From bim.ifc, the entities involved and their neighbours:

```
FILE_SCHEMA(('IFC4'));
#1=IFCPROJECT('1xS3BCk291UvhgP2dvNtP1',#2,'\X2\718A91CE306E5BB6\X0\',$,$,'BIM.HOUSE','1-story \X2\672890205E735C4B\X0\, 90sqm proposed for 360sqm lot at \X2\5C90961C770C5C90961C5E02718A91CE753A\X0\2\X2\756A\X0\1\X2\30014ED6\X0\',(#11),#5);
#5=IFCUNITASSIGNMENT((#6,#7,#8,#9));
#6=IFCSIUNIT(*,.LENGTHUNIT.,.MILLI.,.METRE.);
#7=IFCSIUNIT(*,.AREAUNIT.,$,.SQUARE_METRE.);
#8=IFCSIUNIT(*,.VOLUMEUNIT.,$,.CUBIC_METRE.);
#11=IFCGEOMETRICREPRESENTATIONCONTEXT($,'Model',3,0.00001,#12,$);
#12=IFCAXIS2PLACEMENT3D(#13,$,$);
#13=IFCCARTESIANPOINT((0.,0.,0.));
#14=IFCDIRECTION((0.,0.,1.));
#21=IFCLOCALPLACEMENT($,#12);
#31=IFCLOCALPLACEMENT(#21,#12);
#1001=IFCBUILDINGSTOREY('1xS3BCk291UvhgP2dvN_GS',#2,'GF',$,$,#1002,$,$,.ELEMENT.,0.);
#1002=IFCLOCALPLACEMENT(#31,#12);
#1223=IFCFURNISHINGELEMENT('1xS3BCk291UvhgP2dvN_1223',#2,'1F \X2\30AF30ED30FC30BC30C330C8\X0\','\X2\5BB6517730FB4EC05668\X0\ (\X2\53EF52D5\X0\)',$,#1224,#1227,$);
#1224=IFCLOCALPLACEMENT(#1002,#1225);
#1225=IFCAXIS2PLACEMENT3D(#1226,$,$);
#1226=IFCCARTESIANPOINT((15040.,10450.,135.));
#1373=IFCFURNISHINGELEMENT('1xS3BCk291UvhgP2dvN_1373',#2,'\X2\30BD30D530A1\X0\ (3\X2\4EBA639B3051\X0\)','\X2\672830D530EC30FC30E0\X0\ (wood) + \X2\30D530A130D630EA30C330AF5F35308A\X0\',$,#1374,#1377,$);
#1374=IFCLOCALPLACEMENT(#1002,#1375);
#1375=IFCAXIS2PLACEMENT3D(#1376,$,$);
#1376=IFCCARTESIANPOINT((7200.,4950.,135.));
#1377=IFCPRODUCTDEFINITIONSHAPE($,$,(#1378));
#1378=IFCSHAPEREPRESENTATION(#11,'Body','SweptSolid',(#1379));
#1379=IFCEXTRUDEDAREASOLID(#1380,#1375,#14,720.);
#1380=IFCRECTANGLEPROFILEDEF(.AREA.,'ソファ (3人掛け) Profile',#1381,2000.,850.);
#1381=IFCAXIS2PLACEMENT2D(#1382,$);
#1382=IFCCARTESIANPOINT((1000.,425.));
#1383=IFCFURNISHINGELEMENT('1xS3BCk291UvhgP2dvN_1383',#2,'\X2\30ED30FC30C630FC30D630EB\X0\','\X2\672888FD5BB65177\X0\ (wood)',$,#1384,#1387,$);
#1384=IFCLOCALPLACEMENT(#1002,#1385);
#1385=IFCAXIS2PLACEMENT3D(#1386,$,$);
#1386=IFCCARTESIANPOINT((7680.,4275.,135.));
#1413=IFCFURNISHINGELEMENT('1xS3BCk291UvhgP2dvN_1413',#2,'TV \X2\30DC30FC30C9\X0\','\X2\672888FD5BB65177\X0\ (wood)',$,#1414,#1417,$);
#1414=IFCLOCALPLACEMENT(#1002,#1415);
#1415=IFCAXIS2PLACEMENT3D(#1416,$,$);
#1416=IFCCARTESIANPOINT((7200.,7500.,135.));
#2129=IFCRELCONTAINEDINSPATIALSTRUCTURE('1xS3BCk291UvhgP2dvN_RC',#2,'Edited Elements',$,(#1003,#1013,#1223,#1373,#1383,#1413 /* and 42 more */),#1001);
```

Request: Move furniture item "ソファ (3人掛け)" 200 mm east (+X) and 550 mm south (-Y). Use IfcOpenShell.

```python
import ifcopenshell
import ifcopenshell.api.geometry
import ifcopenshell.util.placement
import ifcopenshell.util.unit

model = ifcopenshell.open("bim.ifc")
unit_scale = ifcopenshell.util.unit.calculate_unit_scale(model)

item = model.by_guid("1xS3BCk291UvhgP2dvN_1373")
matrix = ifcopenshell.util.placement.get_local_placement(item.ObjectPlacement)
matrix[0, 3] += 0.2 / unit_scale
matrix[1, 3] -= 0.55 / unit_scale
ifcopenshell.api.geometry.edit_object_placement(model, product=item, matrix=matrix, is_si=False)

print(ifcopenshell.util.placement.get_local_placement(item.ObjectPlacement).round(3) + 0.0)

model.write("bim_v2.ifc")
```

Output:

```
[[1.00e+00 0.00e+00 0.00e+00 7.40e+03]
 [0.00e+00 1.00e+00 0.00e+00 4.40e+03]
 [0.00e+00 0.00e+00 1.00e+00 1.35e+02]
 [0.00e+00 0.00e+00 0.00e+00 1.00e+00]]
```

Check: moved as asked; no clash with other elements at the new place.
